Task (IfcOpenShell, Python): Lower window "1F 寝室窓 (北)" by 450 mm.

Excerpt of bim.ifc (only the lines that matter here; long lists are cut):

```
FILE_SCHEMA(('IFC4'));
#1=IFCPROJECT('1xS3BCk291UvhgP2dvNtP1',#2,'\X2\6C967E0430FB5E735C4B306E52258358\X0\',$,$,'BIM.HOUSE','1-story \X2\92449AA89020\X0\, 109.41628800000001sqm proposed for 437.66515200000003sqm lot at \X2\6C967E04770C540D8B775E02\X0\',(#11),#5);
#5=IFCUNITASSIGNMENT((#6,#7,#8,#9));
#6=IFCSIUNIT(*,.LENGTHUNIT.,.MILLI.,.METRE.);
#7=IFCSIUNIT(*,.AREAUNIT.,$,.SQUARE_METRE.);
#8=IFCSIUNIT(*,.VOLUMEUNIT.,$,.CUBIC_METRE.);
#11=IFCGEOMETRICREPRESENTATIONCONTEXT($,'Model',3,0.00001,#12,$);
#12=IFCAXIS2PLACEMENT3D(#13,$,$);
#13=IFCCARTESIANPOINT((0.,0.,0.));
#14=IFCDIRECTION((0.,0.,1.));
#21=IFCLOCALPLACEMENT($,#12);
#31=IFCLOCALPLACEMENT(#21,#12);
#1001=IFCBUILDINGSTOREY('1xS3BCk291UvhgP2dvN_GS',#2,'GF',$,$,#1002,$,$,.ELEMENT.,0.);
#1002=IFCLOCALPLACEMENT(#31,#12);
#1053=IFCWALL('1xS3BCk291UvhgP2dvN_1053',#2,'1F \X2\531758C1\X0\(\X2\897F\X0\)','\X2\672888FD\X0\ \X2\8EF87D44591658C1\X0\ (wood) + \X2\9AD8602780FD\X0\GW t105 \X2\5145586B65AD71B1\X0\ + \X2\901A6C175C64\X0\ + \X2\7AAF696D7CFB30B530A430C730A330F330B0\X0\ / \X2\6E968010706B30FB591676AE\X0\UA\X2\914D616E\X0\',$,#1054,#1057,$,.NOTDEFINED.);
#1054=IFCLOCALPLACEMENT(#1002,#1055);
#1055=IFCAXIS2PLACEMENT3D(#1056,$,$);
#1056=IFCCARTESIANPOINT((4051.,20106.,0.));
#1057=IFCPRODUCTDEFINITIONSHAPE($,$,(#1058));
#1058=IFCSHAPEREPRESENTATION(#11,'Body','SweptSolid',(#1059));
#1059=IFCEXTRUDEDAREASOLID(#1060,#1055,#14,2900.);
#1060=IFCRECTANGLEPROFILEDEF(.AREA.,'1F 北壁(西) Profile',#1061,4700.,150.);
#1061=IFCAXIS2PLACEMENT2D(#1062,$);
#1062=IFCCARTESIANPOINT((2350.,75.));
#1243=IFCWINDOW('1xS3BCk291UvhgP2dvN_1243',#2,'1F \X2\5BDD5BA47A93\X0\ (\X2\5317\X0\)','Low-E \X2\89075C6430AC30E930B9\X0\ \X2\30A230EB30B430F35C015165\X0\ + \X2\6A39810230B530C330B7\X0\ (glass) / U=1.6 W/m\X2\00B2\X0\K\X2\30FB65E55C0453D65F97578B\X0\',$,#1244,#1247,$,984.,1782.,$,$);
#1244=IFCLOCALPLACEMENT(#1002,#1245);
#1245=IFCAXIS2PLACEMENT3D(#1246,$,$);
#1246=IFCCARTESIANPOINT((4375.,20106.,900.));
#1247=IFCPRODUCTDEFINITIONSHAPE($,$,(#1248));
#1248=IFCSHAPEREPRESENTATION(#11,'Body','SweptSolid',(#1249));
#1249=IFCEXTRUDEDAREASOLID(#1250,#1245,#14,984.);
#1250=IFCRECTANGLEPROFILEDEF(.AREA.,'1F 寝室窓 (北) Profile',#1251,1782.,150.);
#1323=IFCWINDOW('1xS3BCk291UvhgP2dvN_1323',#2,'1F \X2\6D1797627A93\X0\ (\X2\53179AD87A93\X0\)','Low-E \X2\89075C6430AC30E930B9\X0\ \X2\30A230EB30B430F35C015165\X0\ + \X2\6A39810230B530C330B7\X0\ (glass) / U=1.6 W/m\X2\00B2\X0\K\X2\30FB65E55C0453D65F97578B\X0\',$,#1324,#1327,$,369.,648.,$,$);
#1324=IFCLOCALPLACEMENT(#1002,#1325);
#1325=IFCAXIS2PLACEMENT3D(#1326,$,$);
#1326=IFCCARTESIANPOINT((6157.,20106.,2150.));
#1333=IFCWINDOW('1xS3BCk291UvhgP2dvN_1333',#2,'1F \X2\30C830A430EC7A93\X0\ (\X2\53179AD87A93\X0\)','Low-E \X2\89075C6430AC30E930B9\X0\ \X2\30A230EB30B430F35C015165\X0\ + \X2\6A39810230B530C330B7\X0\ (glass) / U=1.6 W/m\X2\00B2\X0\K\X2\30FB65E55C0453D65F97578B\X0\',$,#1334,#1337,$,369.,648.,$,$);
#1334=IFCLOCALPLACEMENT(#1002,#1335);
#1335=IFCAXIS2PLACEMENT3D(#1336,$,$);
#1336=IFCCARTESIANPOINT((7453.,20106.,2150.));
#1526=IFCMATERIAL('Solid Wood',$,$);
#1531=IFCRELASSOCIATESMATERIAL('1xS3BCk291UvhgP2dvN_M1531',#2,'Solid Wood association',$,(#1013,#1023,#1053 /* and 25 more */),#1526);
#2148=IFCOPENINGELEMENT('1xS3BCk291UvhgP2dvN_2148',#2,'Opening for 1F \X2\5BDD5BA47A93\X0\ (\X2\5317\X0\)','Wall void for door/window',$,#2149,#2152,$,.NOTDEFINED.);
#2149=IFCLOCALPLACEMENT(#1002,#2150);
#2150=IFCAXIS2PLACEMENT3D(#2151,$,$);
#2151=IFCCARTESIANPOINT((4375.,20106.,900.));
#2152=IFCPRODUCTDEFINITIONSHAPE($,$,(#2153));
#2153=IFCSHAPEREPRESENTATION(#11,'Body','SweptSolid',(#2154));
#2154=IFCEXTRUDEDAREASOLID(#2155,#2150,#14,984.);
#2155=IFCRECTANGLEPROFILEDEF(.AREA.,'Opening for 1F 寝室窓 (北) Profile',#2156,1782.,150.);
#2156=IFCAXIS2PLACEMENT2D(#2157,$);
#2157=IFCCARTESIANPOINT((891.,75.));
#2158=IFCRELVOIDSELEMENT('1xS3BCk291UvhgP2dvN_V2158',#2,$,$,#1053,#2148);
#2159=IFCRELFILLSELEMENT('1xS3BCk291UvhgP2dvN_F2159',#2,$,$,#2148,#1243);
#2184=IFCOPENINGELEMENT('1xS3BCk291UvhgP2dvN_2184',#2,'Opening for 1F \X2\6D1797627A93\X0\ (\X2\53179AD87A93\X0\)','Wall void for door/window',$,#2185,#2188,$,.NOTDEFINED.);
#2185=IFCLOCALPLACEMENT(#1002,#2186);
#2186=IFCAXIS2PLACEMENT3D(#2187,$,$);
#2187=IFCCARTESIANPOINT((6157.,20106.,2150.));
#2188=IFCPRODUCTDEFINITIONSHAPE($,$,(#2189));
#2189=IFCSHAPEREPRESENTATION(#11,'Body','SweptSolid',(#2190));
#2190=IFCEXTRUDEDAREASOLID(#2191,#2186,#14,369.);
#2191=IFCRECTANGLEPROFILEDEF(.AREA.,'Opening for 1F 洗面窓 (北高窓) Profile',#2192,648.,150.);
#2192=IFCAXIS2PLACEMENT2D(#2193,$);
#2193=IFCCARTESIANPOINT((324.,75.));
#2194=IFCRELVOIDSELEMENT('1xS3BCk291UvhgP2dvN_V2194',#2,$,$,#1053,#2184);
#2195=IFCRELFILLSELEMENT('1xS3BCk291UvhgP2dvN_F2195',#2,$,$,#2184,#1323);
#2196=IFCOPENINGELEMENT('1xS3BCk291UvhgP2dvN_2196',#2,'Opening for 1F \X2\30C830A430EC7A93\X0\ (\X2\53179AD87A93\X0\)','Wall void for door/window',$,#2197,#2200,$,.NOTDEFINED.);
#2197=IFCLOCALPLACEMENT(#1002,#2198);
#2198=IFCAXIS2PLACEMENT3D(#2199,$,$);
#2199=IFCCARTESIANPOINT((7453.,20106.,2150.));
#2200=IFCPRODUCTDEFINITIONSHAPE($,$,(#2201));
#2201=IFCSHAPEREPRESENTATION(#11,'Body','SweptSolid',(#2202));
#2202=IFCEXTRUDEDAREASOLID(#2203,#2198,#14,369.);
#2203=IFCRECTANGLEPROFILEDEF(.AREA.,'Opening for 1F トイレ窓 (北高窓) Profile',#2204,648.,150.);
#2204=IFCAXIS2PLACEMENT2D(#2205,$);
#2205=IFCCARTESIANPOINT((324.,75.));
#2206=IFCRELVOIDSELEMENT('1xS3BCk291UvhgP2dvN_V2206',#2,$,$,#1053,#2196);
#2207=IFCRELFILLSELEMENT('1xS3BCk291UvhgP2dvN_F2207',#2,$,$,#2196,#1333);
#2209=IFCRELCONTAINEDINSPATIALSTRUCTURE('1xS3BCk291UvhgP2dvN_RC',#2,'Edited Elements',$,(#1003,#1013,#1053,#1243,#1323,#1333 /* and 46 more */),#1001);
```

```python
import numpy as np
import ifcopenshell
import ifcopenshell.api.geometry
import ifcopenshell.util.placement
import ifcopenshell.util.unit

model = ifcopenshell.open("bim.ifc")
unit_scale = ifcopenshell.util.unit.calculate_unit_scale(model)

window = model.by_guid("1xS3BCk291UvhgP2dvN_1243")
opening = window.FillsVoids[0].RelatingOpeningElement
dz = -0.45 / unit_scale

shift = np.array([0.0, 0.0, dz])
# The window is not placed relative to its opening, so move both.
for product in (opening, window):
    matrix = ifcopenshell.util.placement.get_local_placement(product.ObjectPlacement)
    matrix[:3, 3] += shift
    ifcopenshell.api.geometry.edit_object_placement(model, product=product, matrix=matrix, is_si=False)

print(f"moved by {dz * unit_scale:+.3f} m")

model.write("bim_v2.ifc")
```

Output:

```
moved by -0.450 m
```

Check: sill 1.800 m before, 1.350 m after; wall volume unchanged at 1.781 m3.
